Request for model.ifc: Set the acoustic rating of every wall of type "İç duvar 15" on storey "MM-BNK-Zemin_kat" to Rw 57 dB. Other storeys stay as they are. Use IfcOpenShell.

First a look at what the model holds.

```python
import ifcopenshell
import ifcopenshell.util.element

model = ifcopenshell.open("model.ifc")
print(model.schema)
storey = next(s for s in model.by_type("IfcBuildingStorey") if s.Name == "MM-BNK-Zemin_kat")
walls = [e for e in ifcopenshell.util.element.get_decomposition(storey) if e.is_a("IfcWall")]
seen = {}
for e in walls:
    element_type = ifcopenshell.util.element.get_type(e)
    key = (element_type.Name if element_type != e and element_type else None, ifcopenshell.util.element.get_pset(e, "Pset_WallCommon", "AcousticRating"))
    seen[key] = seen.get(key, 0) + 1
for (name, value), count in sorted(seen.items(), key=str):
    print(count, "x", name, "|", value)
```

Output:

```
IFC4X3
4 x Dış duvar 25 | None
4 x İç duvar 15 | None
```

```python
import ifcopenshell
import ifcopenshell.api.pset
import ifcopenshell.util.element

model = ifcopenshell.open("model.ifc")

storey = next(s for s in model.by_type("IfcBuildingStorey") if s.Name == "MM-BNK-Zemin_kat")
walls = [e for e in ifcopenshell.util.element.get_decomposition(storey) if e.is_a("IfcWall")]

count = 0
for e in walls:
    element_type = ifcopenshell.util.element.get_type(e)
    if element_type in (None, e) or element_type.Name != "İç duvar 15":
        continue
    # add_pset returns the element's existing set when there is one.
    pset = ifcopenshell.api.pset.add_pset(model, product=e, name="Pset_WallCommon")
    ifcopenshell.api.pset.edit_pset(model, pset=pset, properties={"AcousticRating": "Rw 57 dB"})
    count += 1

print(count, "walls updated")

model.write("model_edited.ifc")
```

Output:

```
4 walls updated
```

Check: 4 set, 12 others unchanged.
